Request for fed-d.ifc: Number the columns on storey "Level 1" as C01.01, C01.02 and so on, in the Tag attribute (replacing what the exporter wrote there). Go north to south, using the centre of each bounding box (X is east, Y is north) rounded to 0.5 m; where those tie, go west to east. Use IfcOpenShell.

First a look at what the model holds.

```python
import ifcopenshell
import ifcopenshell.util.element
import ifcopenshell.util.placement

model = ifcopenshell.open("fed-d.ifc")
print(model.schema)
storey = next(s for s in model.by_type("IfcBuildingStorey") if s.Name == "Level 1")
columns = [e for e in ifcopenshell.util.element.get_decomposition(storey) if e.is_a("IfcColumn")]
for e in sorted(columns, key=lambda e: e.id()):
    origin = ifcopenshell.util.placement.get_local_placement(e.ObjectPlacement)[:3, 3]
    print(e.id(), e.Tag, e.Name, origin.round(2) + 0.0, sep=" | ")
```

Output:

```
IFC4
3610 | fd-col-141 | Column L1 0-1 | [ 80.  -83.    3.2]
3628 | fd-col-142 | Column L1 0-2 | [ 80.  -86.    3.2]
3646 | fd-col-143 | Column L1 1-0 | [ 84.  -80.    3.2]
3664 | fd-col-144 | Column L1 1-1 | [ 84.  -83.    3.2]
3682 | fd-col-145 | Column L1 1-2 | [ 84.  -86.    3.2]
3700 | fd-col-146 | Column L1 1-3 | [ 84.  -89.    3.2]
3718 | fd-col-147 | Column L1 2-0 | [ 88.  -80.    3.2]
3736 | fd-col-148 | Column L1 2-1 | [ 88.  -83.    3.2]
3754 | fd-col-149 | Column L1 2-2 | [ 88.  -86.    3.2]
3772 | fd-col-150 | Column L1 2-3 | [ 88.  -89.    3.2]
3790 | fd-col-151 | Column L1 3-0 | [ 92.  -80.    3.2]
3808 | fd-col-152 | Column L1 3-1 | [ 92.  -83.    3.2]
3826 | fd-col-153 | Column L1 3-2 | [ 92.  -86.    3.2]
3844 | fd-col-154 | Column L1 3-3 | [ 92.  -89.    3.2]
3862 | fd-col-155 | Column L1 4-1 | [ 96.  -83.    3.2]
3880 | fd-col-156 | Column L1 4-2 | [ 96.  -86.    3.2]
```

```python
import ifcopenshell
import ifcopenshell.geom
import ifcopenshell.util.element
import ifcopenshell.util.shape

model = ifcopenshell.open("fed-d.ifc")
settings = ifcopenshell.geom.settings()
settings.set("use-world-coords", True)


def centre(element):
    shape = ifcopenshell.geom.create_shape(settings, element)
    return ifcopenshell.util.shape.get_bbox_centroid(shape.geometry)


storey = next(s for s in model.by_type("IfcBuildingStorey") if s.Name == "Level 1")
columns = [e for e in ifcopenshell.util.element.get_decomposition(storey) if e.is_a("IfcColumn")]

# Insertion points can sit at a corner or the storey origin, so sort by the geometry (in metres).
centres = {e: centre(e) for e in columns}
columns.sort(key=lambda e: (-round(centres[e][1] / 0.5), centres[e][0]))

for i, e in enumerate(columns, start=1):
    number = f"C01.{i:02d}"
    e.Tag = number
    print(e.id(), number)

model.write("fed-d_edited.ifc")
```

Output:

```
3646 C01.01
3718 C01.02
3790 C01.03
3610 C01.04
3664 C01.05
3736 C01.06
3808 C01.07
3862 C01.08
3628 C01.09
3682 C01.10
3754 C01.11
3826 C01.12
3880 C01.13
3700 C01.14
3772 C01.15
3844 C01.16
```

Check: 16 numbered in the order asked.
